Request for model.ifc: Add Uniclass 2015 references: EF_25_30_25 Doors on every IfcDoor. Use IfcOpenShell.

First a look at what the model holds.

```python
import ifcopenshell

model = ifcopenshell.open("model.ifc")
print(model.schema)
print("classifications:", [c.Name for c in model.by_type("IfcClassification")])
for ifc_class in ("IfcDoor", "IfcRoof", "IfcStair", "IfcWall", "IfcWindow"):
    print(ifc_class, len(model.by_type(ifc_class)))
```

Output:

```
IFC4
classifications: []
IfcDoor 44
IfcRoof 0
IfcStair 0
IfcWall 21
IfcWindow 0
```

```python
import ifcopenshell
import ifcopenshell.api.classification

model = ifcopenshell.open("model.ifc")

system = ifcopenshell.api.classification.add_classification(model, classification="Uniclass 2015")

codes = {
    "IfcDoor": ("EF_25_30_25", "Doors"),
}
for ifc_class, (code, name) in codes.items():
    products = model.by_type(ifc_class)
    ifcopenshell.api.classification.add_reference(
        model, products=products, classification=system, identification=code, name=name
    )
    print(code, len(products))

model.write("model-out.ifc")
```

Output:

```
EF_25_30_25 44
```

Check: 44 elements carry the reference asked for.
